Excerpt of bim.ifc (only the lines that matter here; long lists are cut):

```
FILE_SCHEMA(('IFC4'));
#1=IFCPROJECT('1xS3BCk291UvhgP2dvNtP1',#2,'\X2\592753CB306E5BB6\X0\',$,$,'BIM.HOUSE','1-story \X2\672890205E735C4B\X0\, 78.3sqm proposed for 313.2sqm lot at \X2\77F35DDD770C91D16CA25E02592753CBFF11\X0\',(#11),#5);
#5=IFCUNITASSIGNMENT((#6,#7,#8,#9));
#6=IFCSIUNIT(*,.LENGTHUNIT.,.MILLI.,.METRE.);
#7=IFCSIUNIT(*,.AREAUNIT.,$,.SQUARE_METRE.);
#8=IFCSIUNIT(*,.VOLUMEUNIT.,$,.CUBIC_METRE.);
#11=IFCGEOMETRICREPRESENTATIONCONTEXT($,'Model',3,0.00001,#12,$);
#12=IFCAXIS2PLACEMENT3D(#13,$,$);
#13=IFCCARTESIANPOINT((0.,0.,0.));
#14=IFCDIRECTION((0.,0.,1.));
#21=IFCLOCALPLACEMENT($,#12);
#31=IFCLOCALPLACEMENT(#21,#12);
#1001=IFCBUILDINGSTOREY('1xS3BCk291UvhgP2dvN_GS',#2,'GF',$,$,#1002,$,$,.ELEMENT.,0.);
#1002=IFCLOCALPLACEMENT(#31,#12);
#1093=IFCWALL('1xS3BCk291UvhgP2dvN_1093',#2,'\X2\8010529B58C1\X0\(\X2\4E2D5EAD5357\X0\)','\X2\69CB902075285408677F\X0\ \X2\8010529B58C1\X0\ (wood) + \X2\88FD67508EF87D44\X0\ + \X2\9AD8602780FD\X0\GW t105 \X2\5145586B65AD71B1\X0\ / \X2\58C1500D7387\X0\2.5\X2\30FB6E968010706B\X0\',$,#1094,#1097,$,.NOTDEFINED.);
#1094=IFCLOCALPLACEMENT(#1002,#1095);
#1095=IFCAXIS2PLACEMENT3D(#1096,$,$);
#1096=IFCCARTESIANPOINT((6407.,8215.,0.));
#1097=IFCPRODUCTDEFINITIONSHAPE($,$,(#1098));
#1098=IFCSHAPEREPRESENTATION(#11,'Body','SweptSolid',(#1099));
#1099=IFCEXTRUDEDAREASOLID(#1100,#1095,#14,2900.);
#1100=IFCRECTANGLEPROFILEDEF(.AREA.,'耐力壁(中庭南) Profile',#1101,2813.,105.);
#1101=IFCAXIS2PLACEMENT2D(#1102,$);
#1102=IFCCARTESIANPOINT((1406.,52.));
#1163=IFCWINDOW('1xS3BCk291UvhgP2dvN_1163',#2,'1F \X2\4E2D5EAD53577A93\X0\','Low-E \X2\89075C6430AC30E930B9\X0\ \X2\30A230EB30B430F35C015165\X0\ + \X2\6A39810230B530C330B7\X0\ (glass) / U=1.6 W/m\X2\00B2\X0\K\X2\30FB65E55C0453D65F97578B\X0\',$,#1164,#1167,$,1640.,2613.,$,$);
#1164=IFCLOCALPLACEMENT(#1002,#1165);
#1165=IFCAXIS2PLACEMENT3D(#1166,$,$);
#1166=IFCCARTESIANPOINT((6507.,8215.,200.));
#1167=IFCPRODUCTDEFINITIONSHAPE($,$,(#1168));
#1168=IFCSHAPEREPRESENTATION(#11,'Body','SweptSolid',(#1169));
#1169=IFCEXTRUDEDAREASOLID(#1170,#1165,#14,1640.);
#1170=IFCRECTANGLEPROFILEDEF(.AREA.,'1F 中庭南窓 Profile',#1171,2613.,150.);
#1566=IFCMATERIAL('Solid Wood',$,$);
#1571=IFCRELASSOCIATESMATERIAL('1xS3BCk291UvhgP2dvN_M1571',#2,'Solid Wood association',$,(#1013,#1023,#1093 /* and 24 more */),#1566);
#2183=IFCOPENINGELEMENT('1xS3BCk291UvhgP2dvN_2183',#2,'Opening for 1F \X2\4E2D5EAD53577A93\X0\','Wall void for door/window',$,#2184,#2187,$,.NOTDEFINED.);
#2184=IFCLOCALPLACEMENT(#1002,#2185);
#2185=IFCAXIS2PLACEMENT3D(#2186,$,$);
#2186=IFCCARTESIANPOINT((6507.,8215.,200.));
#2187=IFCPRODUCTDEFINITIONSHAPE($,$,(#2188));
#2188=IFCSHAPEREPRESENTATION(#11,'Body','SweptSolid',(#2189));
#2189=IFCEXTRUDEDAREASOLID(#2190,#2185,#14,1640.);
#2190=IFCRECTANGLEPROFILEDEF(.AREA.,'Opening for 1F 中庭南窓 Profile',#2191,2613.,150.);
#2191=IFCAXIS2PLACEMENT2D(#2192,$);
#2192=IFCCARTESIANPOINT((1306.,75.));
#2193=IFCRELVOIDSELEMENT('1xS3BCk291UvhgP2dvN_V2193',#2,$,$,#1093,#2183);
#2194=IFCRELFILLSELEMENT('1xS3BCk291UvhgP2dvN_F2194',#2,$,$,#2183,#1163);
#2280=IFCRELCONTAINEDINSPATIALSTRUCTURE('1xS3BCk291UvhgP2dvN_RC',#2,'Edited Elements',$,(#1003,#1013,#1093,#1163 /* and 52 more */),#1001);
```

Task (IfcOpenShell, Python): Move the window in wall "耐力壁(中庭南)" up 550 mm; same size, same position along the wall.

```python
import numpy as np
import ifcopenshell
import ifcopenshell.api.geometry
import ifcopenshell.util.placement
import ifcopenshell.util.unit

model = ifcopenshell.open("bim.ifc")
unit_scale = ifcopenshell.util.unit.calculate_unit_scale(model)

window = model.by_guid("1xS3BCk291UvhgP2dvN_1163")
opening = window.FillsVoids[0].RelatingOpeningElement
dz = 0.55 / unit_scale

shift = np.array([0.0, 0.0, dz])
# The window is not placed relative to its opening, so move both.
for product in (opening, window):
    matrix = ifcopenshell.util.placement.get_local_placement(product.ObjectPlacement)
    matrix[:3, 3] += shift
    ifcopenshell.api.geometry.edit_object_placement(model, product=product, matrix=matrix, is_si=False)

print(f"moved by {dz * unit_scale:+.3f} m")

model.write("bim_edited.ifc")
```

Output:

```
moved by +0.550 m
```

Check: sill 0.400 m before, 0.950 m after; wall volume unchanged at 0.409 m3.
